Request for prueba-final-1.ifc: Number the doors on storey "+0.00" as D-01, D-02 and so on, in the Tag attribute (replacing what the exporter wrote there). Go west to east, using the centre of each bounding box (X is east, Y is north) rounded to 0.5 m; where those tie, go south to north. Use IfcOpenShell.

First a look at what the model holds.

```python
import ifcopenshell
import ifcopenshell.util.element
import ifcopenshell.util.placement

model = ifcopenshell.open("prueba-final-1.ifc")
print(model.schema)
storey = next(s for s in model.by_type("IfcBuildingStorey") if s.Name == "+0.00")
doors = [e for e in ifcopenshell.util.element.get_decomposition(storey) if e.is_a("IfcDoor")]
for e in sorted(doors, key=lambda e: e.id()):
    origin = ifcopenshell.util.placement.get_local_placement(e.ObjectPlacement)[:3, 3]
    print(e.id(), e.Tag, e.Name, origin.round(2) + 0.0, sep=" | ")
```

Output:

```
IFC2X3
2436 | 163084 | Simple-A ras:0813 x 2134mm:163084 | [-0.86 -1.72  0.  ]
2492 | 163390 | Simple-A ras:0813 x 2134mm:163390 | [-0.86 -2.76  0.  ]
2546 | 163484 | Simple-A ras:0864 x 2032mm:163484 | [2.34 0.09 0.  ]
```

```python
import ifcopenshell
import ifcopenshell.geom
import ifcopenshell.util.element
import ifcopenshell.util.shape

model = ifcopenshell.open("prueba-final-1.ifc")
settings = ifcopenshell.geom.settings()
settings.set("use-world-coords", True)


def centre(element):
    shape = ifcopenshell.geom.create_shape(settings, element)
    return ifcopenshell.util.shape.get_bbox_centroid(shape.geometry)


storey = next(s for s in model.by_type("IfcBuildingStorey") if s.Name == "+0.00")
doors = [e for e in ifcopenshell.util.element.get_decomposition(storey) if e.is_a("IfcDoor")]

# Insertion points can sit at a corner or the storey origin, so sort by the geometry (in metres).
centres = {e: centre(e) for e in doors}
doors.sort(key=lambda e: (round(centres[e][0] / 0.5), centres[e][1]))

for i, e in enumerate(doors, start=1):
    number = f"D-{i:02d}"
    e.Tag = number
    print(e.id(), number)

model.write("prueba-final-1_updated.ifc")
```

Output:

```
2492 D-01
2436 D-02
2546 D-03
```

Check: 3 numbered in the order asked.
